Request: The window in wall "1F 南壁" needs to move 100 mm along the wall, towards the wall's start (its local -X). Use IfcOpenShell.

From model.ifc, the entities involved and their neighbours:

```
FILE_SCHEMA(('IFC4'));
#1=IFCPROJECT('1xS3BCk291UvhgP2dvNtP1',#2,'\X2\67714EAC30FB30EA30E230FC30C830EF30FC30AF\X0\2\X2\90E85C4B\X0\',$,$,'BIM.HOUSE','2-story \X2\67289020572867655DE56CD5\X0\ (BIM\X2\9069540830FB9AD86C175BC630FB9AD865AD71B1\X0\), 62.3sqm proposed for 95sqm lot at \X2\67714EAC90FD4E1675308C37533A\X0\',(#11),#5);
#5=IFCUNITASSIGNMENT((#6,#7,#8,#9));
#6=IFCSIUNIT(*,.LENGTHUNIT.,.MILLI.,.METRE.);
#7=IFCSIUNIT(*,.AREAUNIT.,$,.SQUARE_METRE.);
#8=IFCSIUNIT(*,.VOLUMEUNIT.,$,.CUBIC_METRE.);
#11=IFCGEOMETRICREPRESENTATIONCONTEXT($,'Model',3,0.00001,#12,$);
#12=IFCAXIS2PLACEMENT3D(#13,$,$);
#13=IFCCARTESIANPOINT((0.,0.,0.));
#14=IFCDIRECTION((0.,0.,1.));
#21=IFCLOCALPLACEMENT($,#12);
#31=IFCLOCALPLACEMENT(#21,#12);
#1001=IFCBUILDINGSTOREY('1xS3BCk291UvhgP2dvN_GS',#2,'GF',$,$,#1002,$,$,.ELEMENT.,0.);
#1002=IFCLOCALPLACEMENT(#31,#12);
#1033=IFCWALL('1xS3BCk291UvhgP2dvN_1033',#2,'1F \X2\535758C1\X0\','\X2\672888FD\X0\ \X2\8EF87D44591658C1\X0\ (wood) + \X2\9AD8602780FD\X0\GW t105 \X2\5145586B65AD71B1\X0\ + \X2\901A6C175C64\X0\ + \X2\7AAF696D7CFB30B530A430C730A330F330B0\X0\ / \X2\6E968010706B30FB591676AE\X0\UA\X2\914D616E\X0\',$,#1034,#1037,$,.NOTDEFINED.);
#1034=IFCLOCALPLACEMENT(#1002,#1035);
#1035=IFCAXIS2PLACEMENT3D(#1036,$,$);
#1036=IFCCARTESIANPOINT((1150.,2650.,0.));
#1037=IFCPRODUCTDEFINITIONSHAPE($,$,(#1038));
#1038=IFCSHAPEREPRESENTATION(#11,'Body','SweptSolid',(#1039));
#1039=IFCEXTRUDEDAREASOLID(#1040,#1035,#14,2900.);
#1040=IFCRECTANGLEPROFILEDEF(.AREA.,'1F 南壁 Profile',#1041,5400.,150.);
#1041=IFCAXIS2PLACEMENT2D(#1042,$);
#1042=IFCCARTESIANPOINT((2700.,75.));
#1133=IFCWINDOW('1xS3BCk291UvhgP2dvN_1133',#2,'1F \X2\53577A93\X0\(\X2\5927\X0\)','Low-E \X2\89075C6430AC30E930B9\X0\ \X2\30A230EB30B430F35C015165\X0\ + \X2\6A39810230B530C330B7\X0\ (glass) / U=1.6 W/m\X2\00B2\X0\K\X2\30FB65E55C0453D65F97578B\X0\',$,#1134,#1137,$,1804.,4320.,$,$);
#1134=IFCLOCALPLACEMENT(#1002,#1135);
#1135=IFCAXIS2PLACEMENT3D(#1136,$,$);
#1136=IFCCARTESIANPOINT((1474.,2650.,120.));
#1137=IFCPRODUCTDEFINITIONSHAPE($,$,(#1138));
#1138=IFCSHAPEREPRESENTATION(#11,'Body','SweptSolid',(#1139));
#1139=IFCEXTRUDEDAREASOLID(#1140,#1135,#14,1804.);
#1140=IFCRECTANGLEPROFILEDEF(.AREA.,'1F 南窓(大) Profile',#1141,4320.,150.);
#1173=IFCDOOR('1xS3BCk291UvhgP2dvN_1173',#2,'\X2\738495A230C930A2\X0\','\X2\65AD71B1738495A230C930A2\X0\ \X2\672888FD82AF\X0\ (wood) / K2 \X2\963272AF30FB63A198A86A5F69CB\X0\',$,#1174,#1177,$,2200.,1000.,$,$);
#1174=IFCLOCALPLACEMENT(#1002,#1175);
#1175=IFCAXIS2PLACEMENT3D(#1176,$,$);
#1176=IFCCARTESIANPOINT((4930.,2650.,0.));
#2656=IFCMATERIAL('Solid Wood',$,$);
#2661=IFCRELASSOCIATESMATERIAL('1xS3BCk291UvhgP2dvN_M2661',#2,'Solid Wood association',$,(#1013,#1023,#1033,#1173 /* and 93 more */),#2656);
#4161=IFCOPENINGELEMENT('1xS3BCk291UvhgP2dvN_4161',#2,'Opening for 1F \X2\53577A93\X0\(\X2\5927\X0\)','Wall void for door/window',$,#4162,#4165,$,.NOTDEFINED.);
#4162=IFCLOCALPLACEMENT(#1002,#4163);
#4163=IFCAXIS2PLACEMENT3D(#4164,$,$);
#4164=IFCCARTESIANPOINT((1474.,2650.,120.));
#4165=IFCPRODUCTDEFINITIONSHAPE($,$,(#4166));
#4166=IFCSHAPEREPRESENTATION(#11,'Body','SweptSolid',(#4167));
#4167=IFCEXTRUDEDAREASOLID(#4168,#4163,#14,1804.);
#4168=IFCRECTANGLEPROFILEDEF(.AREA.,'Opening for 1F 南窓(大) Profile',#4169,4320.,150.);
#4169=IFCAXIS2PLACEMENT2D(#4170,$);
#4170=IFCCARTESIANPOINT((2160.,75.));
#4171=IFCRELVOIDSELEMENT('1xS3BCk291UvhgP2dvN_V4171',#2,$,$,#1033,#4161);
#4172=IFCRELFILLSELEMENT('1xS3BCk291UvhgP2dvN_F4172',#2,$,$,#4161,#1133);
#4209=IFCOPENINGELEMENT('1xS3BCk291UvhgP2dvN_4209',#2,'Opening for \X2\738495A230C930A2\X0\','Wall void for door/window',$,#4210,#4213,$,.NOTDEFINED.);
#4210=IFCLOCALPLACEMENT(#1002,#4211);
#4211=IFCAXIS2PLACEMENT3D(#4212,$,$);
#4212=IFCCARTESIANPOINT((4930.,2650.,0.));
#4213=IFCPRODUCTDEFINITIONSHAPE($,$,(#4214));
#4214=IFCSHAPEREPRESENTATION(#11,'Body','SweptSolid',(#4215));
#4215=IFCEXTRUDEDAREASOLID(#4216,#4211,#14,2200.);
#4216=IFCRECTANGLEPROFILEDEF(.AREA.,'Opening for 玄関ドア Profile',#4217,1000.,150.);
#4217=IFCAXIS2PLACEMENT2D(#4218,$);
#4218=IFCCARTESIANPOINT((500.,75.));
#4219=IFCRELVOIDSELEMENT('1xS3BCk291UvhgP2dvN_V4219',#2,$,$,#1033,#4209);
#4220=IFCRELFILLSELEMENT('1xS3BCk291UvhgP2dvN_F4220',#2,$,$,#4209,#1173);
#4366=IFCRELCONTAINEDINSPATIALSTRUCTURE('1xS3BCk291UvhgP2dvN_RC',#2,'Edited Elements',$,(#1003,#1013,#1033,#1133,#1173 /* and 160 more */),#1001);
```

```python
import ifcopenshell
import ifcopenshell.api.geometry
import ifcopenshell.util.placement

model = ifcopenshell.open("model.ifc")

window = model.by_guid("1xS3BCk291UvhgP2dvN_1133")
opening = window.FillsVoids[0].RelatingOpeningElement
wall = opening.VoidsElements[0].RelatingBuildingElement

wall_matrix = ifcopenshell.util.placement.get_local_placement(wall.ObjectPlacement)
shift = wall_matrix[:3, 0] * -100.0
before = ifcopenshell.util.placement.get_local_placement(window.ObjectPlacement)[:3, 3].copy()

# The window is not placed relative to its opening, so move both.
for product in (opening, window):
    matrix = ifcopenshell.util.placement.get_local_placement(product.ObjectPlacement)
    matrix[:3, 3] += shift
    ifcopenshell.api.geometry.edit_object_placement(model, product=product, matrix=matrix, is_si=False)

after = ifcopenshell.util.placement.get_local_placement(window.ObjectPlacement)[:3, 3]
print("window moved by", (after - before).round(3) + 0.0)

model.write("model_edited.ifc")
```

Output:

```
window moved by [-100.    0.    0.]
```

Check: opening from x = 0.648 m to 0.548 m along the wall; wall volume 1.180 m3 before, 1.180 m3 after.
